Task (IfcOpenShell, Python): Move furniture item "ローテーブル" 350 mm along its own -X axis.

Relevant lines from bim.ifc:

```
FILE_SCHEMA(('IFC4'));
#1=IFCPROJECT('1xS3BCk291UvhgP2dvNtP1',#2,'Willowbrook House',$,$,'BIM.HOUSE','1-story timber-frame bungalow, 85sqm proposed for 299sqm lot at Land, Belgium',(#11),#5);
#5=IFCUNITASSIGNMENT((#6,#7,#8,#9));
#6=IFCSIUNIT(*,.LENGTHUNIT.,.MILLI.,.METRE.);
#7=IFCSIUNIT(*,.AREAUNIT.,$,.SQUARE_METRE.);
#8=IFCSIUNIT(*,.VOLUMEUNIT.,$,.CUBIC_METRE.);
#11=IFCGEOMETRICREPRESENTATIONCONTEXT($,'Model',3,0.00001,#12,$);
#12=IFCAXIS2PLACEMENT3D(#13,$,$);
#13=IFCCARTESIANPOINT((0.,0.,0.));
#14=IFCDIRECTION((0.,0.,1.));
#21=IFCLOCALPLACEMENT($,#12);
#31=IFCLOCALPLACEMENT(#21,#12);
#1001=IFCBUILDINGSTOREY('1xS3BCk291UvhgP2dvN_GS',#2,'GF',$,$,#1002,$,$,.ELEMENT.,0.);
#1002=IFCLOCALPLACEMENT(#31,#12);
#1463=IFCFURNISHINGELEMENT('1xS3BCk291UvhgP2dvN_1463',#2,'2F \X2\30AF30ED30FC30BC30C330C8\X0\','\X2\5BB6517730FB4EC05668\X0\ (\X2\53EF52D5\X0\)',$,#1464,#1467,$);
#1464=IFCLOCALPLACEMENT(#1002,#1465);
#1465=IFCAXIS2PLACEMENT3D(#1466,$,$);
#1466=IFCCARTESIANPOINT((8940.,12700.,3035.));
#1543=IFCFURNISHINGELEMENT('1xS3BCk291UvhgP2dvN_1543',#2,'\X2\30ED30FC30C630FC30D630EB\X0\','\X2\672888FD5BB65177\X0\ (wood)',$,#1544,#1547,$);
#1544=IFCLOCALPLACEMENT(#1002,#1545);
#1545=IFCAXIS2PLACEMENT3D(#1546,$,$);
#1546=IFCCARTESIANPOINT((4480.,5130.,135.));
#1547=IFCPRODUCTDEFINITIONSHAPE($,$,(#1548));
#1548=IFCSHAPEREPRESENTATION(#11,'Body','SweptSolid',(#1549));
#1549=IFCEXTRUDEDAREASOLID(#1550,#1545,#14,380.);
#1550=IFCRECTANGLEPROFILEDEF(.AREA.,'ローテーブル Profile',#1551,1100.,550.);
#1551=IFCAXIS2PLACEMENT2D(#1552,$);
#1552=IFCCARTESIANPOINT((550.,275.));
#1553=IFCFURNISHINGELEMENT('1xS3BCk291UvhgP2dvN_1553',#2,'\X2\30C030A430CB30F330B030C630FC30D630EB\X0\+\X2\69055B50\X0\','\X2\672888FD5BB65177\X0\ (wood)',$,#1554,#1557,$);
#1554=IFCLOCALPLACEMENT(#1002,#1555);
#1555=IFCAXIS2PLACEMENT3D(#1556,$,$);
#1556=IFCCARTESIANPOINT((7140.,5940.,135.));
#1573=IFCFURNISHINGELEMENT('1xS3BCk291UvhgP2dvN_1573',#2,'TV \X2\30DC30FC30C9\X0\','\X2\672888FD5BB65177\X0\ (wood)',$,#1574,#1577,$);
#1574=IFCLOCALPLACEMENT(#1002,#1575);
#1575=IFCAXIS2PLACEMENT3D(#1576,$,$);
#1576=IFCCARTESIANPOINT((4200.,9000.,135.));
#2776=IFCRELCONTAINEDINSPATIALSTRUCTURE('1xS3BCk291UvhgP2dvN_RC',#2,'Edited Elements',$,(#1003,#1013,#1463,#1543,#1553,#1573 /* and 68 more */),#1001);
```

```python
import ifcopenshell
import ifcopenshell.api.geometry
import ifcopenshell.util.placement

model = ifcopenshell.open("bim.ifc")

item = model.by_guid("1xS3BCk291UvhgP2dvN_1543")
matrix = ifcopenshell.util.placement.get_local_placement(item.ObjectPlacement)
matrix[:3, 3] -= matrix[:3, 0] * 350.0
ifcopenshell.api.geometry.edit_object_placement(model, product=item, matrix=matrix, is_si=False)

print(ifcopenshell.util.placement.get_local_placement(item.ObjectPlacement).round(3) + 0.0)

model.write("bim-out.ifc")
```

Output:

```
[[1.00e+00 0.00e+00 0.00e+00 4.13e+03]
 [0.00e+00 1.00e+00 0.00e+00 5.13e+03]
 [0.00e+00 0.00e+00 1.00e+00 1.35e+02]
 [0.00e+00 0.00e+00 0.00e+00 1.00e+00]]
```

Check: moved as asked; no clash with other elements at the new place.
